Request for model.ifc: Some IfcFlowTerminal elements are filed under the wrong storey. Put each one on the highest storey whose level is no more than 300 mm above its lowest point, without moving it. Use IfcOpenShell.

First a look at what the model holds.

```python
import ifcopenshell
import ifcopenshell.util.element
import ifcopenshell.util.placement

model = ifcopenshell.open("model.ifc")
print(model.schema)
for storey in model.by_type("IfcBuildingStorey"):
    level = ifcopenshell.util.placement.get_storey_elevation(storey)
    count = sum(e.is_a("IfcFlowTerminal") for e in ifcopenshell.util.element.get_contained(storey))
    print(storey.id(), storey.Name, round(level, 3), count, sep=" | ")
```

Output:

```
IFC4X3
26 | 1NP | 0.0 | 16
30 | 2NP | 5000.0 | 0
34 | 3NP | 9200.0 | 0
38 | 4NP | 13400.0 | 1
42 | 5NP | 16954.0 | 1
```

```python
import ifcopenshell
import ifcopenshell.api.spatial
import ifcopenshell.geom
import ifcopenshell.util.element
import ifcopenshell.util.placement
import ifcopenshell.util.shape
import ifcopenshell.util.unit

model = ifcopenshell.open("model.ifc")
unit_scale = ifcopenshell.util.unit.calculate_unit_scale(model)
settings = ifcopenshell.geom.settings()

levels = sorted(
    ((ifcopenshell.util.placement.get_storey_elevation(s) * unit_scale, s) for s in model.by_type("IfcBuildingStorey")),
    key=lambda pair: pair[0],
)

for e in model.by_type("IfcFlowTerminal"):
    current = e.ContainedInStructure[0].RelatingStructure if e.ContainedInStructure else None
    if current is None or not current.is_a("IfcBuildingStorey"):
        continue
    shape = ifcopenshell.geom.create_shape(settings, e)
    bottom = ifcopenshell.util.shape.get_shape_bottom_elevation(shape, shape.geometry)
    below = [s for level, s in levels if level <= bottom + 0.3]
    storey = below[-1] if below else levels[0][1]
    if storey != current:
        # assign_container keeps the world position.
        ifcopenshell.api.spatial.assign_container(model, products=[e], relating_structure=storey)
        print(e.id(), current.Name, "->", storey.Name)

model.write("model-out.ifc")
```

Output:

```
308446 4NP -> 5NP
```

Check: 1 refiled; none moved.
